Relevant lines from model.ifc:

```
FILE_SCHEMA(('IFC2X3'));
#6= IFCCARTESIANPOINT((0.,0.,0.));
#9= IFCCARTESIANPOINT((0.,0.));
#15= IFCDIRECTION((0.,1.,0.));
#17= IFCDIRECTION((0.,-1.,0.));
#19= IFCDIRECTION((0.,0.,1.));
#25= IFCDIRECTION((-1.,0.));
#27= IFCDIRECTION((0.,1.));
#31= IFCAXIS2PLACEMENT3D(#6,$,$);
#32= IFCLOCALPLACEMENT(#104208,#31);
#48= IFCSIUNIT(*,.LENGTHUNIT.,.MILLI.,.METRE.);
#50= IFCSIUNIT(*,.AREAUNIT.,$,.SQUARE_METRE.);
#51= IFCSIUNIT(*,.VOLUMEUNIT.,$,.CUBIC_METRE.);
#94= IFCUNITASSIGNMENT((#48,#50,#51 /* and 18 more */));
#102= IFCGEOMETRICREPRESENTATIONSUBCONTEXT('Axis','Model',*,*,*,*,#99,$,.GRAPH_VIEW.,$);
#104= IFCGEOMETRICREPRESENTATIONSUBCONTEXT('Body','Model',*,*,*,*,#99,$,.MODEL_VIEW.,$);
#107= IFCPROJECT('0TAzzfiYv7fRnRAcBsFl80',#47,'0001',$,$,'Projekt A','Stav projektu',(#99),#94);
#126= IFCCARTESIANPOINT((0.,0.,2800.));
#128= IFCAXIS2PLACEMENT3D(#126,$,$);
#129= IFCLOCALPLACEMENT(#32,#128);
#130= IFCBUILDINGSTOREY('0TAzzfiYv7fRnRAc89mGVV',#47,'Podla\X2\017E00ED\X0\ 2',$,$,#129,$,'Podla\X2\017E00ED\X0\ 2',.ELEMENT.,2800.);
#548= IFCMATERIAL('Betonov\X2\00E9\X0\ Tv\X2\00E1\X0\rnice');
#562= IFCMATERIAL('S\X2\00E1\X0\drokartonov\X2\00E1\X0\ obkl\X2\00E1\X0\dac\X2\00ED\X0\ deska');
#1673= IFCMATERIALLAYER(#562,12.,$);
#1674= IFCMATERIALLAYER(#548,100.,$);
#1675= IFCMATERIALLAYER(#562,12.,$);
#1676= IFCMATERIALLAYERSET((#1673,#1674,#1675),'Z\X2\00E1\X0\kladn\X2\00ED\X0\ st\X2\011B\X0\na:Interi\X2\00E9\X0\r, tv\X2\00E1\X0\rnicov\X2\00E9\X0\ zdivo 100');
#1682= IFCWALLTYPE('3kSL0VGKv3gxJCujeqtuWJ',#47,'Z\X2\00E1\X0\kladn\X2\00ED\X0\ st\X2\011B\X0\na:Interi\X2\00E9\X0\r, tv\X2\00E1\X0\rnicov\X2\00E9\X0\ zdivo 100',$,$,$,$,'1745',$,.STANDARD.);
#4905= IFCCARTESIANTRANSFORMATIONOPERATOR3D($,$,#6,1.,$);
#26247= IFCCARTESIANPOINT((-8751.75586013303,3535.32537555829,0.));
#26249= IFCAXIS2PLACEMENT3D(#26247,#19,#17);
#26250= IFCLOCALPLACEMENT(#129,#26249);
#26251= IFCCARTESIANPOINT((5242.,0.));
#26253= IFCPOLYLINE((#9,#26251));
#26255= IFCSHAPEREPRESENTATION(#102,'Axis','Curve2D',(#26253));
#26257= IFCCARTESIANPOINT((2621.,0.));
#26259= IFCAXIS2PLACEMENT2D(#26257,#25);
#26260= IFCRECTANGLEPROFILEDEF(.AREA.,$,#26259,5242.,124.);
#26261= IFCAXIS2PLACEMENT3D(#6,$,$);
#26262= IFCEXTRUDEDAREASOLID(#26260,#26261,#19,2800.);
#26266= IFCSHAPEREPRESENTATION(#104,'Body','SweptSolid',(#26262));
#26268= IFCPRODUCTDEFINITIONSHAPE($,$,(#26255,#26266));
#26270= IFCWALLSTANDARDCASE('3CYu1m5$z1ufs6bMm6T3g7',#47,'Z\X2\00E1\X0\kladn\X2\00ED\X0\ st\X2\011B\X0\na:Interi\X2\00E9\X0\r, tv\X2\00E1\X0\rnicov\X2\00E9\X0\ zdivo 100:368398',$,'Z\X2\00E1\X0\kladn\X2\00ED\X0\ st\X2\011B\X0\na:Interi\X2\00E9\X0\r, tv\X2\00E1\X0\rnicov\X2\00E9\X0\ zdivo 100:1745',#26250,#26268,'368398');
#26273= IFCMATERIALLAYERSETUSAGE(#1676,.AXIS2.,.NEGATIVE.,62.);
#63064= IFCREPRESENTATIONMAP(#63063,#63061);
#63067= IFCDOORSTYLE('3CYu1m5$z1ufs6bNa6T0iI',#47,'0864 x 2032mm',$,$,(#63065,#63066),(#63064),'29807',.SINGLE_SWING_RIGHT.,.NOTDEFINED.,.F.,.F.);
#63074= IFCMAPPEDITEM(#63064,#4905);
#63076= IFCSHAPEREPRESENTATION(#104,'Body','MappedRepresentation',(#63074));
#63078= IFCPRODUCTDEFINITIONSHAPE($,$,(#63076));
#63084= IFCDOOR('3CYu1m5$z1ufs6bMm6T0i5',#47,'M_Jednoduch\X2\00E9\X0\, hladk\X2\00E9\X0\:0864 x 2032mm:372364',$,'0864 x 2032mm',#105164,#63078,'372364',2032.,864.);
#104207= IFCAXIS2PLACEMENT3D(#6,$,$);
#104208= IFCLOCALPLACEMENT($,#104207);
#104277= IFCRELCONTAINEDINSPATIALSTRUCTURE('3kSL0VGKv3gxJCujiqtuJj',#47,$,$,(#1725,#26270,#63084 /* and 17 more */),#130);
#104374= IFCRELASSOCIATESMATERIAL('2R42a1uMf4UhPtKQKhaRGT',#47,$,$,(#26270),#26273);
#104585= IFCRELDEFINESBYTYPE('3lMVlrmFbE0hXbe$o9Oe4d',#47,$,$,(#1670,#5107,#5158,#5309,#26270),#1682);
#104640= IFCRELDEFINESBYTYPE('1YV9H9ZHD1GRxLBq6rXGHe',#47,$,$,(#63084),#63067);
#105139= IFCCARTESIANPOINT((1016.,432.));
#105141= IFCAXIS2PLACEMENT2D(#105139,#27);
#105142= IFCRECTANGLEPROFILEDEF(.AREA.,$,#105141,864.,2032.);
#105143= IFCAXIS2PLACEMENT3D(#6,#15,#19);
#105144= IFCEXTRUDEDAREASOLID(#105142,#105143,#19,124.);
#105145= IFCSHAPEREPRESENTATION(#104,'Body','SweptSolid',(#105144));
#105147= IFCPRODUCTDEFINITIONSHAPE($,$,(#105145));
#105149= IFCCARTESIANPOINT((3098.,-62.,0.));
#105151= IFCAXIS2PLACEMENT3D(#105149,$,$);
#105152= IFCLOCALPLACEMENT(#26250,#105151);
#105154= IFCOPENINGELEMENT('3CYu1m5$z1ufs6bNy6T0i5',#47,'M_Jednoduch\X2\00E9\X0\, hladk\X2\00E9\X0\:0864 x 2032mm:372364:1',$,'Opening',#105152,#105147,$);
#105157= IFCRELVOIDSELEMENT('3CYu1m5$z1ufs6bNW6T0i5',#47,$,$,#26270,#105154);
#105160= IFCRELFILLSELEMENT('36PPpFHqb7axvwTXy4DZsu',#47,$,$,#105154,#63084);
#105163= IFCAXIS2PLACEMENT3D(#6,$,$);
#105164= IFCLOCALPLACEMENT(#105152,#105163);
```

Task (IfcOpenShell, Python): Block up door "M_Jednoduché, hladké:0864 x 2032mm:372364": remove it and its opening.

```python
import ifcopenshell
import ifcopenshell.api.feature
import ifcopenshell.api.root
import ifcopenshell.geom
import ifcopenshell.util.shape

model = ifcopenshell.open("model.ifc")
settings = ifcopenshell.geom.settings()


def volume(element):
    """Net volume in cubic metres, openings subtracted."""
    shape = ifcopenshell.geom.create_shape(settings, element)
    return ifcopenshell.util.shape.get_volume(shape.geometry)


door = model.by_guid("3CYu1m5$z1ufs6bMm6T0i5")
opening = door.FillsVoids[0].RelatingOpeningElement
wall = opening.VoidsElements[0].RelatingBuildingElement
before = volume(wall)

ifcopenshell.api.root.remove_product(model, product=door)
ifcopenshell.api.feature.remove_feature(model, feature=opening)

after = volume(wall)

print(f"wall volume {before:.3f} -> {after:.3f} m3")

model.write("model_edited.ifc")
```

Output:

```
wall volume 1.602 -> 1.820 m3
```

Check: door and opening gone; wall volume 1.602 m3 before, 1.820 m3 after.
